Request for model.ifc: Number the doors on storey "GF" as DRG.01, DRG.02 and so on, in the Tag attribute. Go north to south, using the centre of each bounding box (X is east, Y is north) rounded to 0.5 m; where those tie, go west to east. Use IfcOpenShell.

First a look at what the model holds.

```python
import ifcopenshell
import ifcopenshell.util.element
import ifcopenshell.util.placement

model = ifcopenshell.open("model.ifc")
print(model.schema)
storey = next(s for s in model.by_type("IfcBuildingStorey") if s.Name == "GF")
doors = [e for e in ifcopenshell.util.element.get_decomposition(storey) if e.is_a("IfcDoor")]
for e in sorted(doors, key=lambda e: e.id()):
    origin = ifcopenshell.util.placement.get_local_placement(e.ObjectPlacement)[:3, 3]
    print(e.id(), e.Tag, e.Name, origin.round(2) + 0.0, sep=" | ")
```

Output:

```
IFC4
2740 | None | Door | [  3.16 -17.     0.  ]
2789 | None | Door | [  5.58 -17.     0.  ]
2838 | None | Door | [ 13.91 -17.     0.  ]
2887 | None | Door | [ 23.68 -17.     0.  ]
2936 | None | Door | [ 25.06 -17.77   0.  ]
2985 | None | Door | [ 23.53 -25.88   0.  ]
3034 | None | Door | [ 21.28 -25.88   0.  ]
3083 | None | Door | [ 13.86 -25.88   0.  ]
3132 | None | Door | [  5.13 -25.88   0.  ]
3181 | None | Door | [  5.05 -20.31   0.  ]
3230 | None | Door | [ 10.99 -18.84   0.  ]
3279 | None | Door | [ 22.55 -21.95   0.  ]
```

```python
import ifcopenshell
import ifcopenshell.geom
import ifcopenshell.util.element
import ifcopenshell.util.shape

model = ifcopenshell.open("model.ifc")
settings = ifcopenshell.geom.settings()
settings.set("use-world-coords", True)


def centre(element):
    shape = ifcopenshell.geom.create_shape(settings, element)
    return ifcopenshell.util.shape.get_bbox_centroid(shape.geometry)


storey = next(s for s in model.by_type("IfcBuildingStorey") if s.Name == "GF")
doors = [e for e in ifcopenshell.util.element.get_decomposition(storey) if e.is_a("IfcDoor")]

# Insertion points can sit at a corner or the storey origin, so sort by the geometry (in metres).
centres = {e: centre(e) for e in doors}
doors.sort(key=lambda e: (-round(centres[e][1] / 0.5), centres[e][0]))

for i, e in enumerate(doors, start=1):
    number = f"DRG.{i:02d}"
    e.Tag = number
    print(e.id(), number)

model.write("model-out.ifc")
```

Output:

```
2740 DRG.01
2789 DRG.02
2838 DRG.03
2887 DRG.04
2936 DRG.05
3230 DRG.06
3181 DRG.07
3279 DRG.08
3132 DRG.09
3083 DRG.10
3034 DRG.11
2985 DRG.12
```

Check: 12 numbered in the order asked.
